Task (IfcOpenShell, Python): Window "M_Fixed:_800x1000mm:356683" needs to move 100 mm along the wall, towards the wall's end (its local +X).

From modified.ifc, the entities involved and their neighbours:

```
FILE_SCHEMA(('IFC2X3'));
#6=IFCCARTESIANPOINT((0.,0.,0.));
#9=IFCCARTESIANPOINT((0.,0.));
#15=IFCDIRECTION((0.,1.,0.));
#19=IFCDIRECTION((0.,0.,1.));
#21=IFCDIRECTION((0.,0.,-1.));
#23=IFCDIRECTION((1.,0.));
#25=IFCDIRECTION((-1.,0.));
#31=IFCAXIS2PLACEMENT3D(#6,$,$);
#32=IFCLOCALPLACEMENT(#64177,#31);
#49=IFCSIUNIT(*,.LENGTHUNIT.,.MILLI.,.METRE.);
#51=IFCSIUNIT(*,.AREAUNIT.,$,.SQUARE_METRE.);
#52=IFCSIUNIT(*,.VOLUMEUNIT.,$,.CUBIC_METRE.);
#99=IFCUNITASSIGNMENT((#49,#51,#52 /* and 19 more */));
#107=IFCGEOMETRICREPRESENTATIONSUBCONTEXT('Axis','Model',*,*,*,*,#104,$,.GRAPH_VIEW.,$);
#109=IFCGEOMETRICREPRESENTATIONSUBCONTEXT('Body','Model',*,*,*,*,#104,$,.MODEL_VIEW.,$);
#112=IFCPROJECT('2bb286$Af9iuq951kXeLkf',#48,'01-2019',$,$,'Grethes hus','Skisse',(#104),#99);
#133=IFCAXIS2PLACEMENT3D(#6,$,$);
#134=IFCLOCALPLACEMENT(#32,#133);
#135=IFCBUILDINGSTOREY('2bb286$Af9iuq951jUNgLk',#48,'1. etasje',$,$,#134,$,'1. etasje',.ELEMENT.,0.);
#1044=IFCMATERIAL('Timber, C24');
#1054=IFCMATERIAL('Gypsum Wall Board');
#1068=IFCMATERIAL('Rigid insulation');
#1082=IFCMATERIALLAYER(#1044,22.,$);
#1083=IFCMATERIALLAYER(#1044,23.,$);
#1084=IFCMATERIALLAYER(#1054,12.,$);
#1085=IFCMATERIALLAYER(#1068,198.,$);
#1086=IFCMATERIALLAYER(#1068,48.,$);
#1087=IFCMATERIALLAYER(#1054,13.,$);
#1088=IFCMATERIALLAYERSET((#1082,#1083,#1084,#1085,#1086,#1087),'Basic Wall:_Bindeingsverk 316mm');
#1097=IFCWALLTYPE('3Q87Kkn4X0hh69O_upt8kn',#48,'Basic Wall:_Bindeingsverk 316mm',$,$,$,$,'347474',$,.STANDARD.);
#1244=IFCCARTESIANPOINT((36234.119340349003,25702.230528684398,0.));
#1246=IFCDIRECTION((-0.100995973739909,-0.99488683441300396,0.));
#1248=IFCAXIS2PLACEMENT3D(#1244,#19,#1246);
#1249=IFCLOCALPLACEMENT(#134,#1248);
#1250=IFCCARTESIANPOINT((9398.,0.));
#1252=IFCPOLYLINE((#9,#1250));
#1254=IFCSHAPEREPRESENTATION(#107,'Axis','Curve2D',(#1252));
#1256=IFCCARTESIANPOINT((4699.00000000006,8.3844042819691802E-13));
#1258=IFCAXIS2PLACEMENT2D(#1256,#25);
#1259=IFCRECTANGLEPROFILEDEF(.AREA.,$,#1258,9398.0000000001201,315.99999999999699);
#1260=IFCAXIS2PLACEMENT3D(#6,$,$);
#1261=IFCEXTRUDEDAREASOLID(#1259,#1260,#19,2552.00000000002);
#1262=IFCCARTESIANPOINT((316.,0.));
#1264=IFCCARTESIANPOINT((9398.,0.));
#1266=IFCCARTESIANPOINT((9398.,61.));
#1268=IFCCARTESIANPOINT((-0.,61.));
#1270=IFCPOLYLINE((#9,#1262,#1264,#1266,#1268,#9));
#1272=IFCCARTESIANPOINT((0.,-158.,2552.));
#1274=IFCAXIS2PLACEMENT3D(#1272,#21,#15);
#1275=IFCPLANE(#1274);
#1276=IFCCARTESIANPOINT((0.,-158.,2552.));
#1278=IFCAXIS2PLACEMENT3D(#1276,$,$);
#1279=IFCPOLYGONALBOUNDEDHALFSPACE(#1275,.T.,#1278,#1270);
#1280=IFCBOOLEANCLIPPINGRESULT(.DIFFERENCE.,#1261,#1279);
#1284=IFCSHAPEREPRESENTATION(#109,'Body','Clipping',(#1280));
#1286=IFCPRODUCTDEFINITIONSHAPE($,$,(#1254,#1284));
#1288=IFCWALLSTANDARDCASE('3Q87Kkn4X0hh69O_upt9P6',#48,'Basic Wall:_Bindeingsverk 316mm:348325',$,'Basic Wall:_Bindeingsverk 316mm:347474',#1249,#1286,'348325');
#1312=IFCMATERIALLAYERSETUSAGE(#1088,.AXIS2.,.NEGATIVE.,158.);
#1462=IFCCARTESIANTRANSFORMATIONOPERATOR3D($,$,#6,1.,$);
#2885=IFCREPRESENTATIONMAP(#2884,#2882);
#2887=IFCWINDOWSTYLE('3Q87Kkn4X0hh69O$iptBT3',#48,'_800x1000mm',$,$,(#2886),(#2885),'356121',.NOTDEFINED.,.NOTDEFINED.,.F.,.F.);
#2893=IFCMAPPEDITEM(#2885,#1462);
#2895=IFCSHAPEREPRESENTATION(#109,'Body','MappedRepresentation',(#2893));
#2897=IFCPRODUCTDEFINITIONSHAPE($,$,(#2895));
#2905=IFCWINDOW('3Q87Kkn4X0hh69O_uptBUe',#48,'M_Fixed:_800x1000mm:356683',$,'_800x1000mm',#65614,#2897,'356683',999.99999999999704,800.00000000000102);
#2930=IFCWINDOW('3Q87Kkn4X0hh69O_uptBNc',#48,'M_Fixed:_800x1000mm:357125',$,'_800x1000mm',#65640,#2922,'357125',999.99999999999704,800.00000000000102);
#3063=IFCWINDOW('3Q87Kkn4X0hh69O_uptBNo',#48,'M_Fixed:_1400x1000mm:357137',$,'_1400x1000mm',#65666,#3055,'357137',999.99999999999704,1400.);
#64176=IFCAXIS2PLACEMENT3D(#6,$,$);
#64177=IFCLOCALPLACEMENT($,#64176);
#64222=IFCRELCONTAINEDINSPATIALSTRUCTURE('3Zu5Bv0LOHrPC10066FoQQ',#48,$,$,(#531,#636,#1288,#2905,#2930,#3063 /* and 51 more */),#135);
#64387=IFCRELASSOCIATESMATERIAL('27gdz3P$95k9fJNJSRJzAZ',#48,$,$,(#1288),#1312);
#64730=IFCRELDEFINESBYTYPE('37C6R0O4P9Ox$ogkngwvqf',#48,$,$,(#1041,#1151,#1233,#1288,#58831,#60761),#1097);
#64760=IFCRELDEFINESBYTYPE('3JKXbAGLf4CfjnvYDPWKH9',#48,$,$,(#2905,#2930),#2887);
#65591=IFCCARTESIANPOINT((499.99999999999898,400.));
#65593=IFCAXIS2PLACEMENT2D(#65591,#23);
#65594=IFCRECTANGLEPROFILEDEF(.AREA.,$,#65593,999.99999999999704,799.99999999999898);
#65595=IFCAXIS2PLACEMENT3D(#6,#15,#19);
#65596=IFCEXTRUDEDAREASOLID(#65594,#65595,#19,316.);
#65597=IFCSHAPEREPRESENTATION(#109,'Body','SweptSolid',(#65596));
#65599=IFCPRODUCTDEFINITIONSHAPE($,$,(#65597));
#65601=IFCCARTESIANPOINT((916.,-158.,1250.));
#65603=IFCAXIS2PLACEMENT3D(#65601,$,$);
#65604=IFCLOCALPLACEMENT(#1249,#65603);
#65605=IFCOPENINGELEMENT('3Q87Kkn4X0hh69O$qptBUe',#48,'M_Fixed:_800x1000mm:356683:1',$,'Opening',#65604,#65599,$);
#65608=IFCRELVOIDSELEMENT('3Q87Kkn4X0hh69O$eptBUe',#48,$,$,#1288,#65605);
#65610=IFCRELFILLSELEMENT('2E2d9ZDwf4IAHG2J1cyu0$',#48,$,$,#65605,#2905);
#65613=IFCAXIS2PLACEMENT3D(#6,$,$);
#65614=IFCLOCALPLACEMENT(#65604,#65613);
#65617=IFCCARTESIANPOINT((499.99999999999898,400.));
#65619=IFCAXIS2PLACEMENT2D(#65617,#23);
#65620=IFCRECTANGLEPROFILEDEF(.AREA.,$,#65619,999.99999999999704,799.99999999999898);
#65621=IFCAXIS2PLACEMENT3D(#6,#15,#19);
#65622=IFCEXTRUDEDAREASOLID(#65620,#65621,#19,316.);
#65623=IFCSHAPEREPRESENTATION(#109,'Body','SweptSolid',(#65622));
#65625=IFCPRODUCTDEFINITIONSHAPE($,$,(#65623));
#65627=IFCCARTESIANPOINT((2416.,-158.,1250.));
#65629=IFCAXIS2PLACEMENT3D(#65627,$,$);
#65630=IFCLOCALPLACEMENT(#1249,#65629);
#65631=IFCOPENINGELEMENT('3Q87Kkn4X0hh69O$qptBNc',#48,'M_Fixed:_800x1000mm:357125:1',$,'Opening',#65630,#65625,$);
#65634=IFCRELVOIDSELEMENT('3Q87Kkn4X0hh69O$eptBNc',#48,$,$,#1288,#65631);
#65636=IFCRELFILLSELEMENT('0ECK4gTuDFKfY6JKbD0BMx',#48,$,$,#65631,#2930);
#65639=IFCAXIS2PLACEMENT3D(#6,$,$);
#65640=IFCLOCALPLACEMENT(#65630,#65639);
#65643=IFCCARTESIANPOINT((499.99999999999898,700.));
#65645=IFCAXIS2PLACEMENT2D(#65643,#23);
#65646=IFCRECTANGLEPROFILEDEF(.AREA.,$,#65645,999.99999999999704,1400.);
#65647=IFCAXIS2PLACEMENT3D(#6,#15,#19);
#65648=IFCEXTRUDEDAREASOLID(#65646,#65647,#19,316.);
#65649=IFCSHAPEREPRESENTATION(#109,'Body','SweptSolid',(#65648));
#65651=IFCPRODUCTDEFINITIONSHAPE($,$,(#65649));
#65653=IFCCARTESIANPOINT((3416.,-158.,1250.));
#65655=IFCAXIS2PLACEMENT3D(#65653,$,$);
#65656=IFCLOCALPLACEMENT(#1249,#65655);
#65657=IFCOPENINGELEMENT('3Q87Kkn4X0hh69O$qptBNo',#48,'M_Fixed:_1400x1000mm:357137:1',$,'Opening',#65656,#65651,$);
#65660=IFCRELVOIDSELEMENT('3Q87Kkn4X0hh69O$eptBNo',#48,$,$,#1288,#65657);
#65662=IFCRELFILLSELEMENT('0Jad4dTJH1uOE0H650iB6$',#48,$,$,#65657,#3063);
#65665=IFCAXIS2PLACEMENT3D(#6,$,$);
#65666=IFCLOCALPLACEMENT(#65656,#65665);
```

```python
import ifcopenshell
import ifcopenshell.api.geometry
import ifcopenshell.util.placement

model = ifcopenshell.open("modified.ifc")

window = model.by_guid("3Q87Kkn4X0hh69O_uptBUe")
opening = window.FillsVoids[0].RelatingOpeningElement
wall = opening.VoidsElements[0].RelatingBuildingElement

wall_matrix = ifcopenshell.util.placement.get_local_placement(wall.ObjectPlacement)
shift = wall_matrix[:3, 0] * 100.0
before = ifcopenshell.util.placement.get_local_placement(window.ObjectPlacement)[:3, 3].copy()

# The window is placed relative to its opening, so it follows when the opening moves.
matrix = ifcopenshell.util.placement.get_local_placement(opening.ObjectPlacement)
matrix[:3, 3] += shift
ifcopenshell.api.geometry.edit_object_placement(
    model, product=opening, matrix=matrix, is_si=False, should_transform_children=True
)

after = ifcopenshell.util.placement.get_local_placement(window.ObjectPlacement)[:3, 3]
print("window moved by", (after - before).round(3) + 0.0)

model.write("modified_v2.ifc")
```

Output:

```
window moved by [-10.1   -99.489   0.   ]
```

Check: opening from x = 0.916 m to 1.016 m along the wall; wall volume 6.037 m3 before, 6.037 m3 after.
